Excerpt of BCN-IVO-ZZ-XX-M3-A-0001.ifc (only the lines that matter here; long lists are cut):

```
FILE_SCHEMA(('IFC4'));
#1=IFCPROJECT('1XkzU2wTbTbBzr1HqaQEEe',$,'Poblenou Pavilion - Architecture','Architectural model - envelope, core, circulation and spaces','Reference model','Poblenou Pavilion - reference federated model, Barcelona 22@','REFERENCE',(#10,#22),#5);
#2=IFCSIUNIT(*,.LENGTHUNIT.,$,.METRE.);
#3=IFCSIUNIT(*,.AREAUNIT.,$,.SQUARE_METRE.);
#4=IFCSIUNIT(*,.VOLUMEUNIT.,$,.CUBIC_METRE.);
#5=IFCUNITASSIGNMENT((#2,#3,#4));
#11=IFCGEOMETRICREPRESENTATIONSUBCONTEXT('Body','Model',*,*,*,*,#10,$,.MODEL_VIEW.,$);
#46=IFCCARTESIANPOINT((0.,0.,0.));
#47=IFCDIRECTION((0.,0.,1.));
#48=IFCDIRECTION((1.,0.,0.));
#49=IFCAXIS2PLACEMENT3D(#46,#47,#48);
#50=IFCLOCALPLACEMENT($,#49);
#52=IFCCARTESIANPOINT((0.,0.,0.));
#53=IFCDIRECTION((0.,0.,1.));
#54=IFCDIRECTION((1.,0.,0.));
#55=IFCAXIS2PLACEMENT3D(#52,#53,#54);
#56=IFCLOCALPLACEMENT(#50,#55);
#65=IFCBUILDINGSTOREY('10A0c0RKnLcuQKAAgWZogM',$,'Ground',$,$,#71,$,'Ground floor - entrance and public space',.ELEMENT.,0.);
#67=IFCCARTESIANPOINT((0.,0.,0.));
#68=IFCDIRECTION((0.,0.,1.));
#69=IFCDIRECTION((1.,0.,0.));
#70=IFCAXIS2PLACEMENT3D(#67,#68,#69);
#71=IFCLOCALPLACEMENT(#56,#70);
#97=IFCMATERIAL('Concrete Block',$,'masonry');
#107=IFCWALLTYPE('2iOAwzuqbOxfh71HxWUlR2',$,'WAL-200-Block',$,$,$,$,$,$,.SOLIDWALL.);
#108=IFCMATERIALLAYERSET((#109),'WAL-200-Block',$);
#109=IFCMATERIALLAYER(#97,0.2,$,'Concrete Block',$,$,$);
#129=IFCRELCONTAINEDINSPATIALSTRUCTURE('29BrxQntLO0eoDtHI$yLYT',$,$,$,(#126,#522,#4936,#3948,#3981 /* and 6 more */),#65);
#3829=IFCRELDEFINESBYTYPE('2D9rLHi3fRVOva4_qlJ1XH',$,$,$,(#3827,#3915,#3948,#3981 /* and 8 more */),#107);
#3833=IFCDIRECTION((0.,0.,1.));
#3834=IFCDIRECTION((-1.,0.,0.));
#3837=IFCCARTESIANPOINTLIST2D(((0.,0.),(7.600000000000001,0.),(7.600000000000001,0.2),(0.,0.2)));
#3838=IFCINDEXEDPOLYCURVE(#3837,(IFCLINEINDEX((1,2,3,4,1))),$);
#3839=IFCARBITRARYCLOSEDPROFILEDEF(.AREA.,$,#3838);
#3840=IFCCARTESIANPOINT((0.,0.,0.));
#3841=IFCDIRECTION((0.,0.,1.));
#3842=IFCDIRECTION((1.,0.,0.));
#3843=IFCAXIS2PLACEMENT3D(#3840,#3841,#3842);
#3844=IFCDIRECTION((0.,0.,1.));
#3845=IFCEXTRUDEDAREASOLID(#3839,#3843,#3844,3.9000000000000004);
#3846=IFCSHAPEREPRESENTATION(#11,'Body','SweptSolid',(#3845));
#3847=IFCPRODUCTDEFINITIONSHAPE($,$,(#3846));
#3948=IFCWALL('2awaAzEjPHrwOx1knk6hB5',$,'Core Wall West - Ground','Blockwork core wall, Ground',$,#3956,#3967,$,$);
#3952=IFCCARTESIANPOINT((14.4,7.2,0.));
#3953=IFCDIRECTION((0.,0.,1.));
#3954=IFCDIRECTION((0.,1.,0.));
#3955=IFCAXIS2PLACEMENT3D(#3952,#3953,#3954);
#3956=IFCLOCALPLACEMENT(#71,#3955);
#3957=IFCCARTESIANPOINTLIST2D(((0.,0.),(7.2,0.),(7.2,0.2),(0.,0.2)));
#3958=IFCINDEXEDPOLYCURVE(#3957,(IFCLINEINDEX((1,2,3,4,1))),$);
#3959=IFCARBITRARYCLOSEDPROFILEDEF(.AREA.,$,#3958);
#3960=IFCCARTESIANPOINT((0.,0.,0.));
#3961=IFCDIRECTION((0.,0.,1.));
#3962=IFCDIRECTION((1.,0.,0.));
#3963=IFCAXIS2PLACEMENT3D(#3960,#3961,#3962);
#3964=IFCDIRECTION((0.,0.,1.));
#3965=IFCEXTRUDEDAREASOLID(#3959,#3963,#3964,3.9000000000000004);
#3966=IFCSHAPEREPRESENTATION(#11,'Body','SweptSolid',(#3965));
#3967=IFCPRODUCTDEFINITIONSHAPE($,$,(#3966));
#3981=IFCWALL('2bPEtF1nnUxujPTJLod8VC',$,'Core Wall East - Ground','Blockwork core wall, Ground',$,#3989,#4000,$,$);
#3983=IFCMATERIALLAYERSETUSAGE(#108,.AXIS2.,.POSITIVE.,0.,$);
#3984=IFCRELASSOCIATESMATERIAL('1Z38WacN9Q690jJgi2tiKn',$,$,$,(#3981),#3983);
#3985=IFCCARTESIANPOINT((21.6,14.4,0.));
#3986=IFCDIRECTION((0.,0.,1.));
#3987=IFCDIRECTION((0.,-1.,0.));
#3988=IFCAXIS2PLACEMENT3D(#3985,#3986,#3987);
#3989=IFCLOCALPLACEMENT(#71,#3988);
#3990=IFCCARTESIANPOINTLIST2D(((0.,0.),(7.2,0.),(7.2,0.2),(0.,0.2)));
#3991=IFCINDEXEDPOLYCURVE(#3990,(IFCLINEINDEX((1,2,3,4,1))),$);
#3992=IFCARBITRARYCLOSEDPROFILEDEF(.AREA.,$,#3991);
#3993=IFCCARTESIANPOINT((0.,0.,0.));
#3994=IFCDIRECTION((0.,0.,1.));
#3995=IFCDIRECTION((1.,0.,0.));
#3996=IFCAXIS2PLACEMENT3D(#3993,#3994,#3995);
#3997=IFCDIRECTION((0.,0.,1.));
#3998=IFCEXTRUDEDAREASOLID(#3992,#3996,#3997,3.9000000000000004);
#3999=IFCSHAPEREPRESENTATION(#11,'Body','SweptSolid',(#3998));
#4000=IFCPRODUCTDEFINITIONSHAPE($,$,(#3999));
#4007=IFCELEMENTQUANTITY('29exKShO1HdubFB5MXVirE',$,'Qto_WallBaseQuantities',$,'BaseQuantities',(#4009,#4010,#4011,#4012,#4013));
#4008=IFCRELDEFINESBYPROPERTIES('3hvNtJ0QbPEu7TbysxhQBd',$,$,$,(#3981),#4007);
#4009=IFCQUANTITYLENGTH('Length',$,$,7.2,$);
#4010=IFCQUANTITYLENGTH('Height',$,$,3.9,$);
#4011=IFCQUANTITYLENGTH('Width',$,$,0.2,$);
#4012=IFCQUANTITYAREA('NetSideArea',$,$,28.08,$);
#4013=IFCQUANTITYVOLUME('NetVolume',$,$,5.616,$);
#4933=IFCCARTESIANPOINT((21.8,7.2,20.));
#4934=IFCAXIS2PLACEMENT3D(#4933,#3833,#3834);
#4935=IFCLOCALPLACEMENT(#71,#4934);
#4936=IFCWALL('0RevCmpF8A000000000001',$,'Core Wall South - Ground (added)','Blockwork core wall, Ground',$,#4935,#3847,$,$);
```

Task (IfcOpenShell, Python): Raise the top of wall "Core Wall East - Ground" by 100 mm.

```python
import ifcopenshell
import ifcopenshell.api.pset
import ifcopenshell.geom
import ifcopenshell.util.element
import ifcopenshell.util.representation
import ifcopenshell.util.shape
import ifcopenshell.util.unit

model = ifcopenshell.open("BCN-IVO-ZZ-XX-M3-A-0001.ifc")
unit_scale = ifcopenshell.util.unit.calculate_unit_scale(model)
area_scale = ifcopenshell.util.unit.calculate_unit_scale(model, "AREAUNIT")
volume_scale = ifcopenshell.util.unit.calculate_unit_scale(model, "VOLUMEUNIT")
settings = ifcopenshell.geom.settings()


def volume(element):
    """Net volume in cubic metres, openings subtracted."""
    shape = ifcopenshell.geom.create_shape(settings, element)
    return ifcopenshell.util.shape.get_volume(shape.geometry)


wall = model.by_guid("2bPEtF1nnUxujPTJLod8VC")
before = volume(wall)

body = ifcopenshell.util.representation.get_representation(wall, "Model", "Body")
solid = body.Items[0]
old_height = solid.Depth
solid.Depth += 0.1 / unit_scale
after = volume(wall)
thickness = 0.2  # wall thickness in metres

# Update the stored height, areas and volumes.
qto = model.by_id(ifcopenshell.util.element.get_pset(wall, "Qto_WallBaseQuantities", should_inherit=False)["id"])
ifcopenshell.api.pset.edit_qto(model, qto=qto, properties={
    "Height": solid.Depth,
    "NetSideArea": after / thickness / area_scale,
    "NetVolume": after / volume_scale,
})

print(f"height {old_height:g} -> {solid.Depth:g}, volume {before:.3f} -> {after:.3f} m3")

model.write("BCN-IVO-ZZ-XX-M3-A-0001_updated.ifc")
```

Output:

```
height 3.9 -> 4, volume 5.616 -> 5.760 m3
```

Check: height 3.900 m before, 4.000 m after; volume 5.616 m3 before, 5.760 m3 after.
